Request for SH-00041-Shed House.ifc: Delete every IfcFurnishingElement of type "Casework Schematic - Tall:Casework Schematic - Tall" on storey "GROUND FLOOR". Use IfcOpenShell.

First a look at what the model holds.

```python
import ifcopenshell
import ifcopenshell.util.element

model = ifcopenshell.open("SH-00041-Shed House.ifc")
print(model.schema)
storey = next(s for s in model.by_type("IfcBuildingStorey") if s.Name == "GROUND FLOOR")
furniture = [e for e in ifcopenshell.util.element.get_decomposition(storey) if e.is_a("IfcFurnishingElement")]
seen = {}
for e in furniture:
    element_type = ifcopenshell.util.element.get_type(e)
    name = element_type.Name if element_type not in (None, e) else None
    seen[name] = seen.get(name, 0) + 1
for name, count in sorted(seen.items(), key=str):
    print(count, "x", name)
```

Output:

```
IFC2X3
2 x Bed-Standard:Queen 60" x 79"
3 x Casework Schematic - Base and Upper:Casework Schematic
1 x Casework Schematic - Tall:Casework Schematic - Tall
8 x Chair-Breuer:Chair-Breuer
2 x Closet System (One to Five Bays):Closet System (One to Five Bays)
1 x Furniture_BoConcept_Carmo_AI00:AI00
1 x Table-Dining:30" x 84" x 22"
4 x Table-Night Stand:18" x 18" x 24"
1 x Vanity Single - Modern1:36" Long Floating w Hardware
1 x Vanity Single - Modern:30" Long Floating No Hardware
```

```python
import ifcopenshell
import ifcopenshell.api.root
import ifcopenshell.util.element

model = ifcopenshell.open("SH-00041-Shed House.ifc")

storey = next(s for s in model.by_type("IfcBuildingStorey") if s.Name == "GROUND FLOOR")
furniture = [e for e in ifcopenshell.util.element.get_decomposition(storey) if e.is_a("IfcFurnishingElement")]
targets = [e for e in furniture if (t := ifcopenshell.util.element.get_type(e)) not in (None, e) and t.Name == "Casework Schematic - Tall:Casework Schematic - Tall"]

for e in targets:
    ifcopenshell.api.root.remove_product(model, product=e)
print(len(targets), "removed")

model.write("SH-00041-Shed House_rev.ifc")
```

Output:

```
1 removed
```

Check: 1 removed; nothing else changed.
